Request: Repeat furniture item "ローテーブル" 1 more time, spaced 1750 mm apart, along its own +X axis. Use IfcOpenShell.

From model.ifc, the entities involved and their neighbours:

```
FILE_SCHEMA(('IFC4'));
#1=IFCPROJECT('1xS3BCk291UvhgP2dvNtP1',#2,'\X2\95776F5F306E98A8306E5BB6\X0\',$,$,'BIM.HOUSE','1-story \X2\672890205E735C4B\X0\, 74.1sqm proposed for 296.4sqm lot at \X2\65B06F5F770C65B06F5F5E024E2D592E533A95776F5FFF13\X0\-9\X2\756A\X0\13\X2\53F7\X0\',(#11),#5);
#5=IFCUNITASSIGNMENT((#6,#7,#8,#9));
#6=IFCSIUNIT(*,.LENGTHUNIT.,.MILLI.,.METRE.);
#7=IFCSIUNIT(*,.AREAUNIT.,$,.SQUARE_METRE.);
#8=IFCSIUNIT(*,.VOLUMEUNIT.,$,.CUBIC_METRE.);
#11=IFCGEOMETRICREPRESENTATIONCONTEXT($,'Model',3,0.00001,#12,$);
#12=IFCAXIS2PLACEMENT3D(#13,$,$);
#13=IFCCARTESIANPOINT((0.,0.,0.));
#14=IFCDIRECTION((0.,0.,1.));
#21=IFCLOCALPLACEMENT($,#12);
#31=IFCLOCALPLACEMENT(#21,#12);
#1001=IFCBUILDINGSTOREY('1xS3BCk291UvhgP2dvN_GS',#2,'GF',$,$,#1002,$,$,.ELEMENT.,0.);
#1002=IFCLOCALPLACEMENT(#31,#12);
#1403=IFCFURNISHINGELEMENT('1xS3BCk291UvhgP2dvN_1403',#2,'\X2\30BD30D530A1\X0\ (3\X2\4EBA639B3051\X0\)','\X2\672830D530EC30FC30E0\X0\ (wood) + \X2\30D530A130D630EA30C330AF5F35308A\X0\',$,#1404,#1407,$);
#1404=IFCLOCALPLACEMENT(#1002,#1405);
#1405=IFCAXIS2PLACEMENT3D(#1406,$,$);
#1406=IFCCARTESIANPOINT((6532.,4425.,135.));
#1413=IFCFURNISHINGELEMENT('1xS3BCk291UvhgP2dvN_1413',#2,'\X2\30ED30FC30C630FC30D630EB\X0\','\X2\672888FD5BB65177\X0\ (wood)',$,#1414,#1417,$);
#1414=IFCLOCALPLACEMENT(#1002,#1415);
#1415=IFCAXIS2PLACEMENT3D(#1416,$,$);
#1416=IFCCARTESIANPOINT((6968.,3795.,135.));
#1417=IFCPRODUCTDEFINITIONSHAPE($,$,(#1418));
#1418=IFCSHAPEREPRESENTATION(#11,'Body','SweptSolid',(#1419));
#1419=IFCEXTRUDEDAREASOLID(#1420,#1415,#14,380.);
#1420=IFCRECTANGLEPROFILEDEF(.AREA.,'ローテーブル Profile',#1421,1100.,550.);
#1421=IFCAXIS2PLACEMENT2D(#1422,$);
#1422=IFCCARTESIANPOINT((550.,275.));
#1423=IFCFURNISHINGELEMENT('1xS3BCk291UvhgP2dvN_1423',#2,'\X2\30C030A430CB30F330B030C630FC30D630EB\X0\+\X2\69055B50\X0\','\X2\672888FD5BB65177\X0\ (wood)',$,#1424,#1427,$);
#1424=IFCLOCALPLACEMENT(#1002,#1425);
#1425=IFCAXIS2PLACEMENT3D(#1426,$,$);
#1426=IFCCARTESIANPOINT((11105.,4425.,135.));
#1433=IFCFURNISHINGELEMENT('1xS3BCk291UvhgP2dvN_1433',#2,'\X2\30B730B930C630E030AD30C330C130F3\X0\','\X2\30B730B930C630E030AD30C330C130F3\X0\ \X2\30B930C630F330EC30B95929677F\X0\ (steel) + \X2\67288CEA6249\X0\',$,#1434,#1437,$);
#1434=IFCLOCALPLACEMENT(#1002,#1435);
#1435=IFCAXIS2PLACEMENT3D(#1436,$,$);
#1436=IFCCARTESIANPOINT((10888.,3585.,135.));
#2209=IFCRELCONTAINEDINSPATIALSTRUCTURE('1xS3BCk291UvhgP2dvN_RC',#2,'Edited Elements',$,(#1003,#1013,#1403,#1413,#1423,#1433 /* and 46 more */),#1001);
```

```python
import ifcopenshell
import ifcopenshell.api.geometry
import ifcopenshell.api.root
import ifcopenshell.util.element
import ifcopenshell.util.placement
import ifcopenshell.util.unit

model = ifcopenshell.open("model.ifc")
unit_scale = ifcopenshell.util.unit.calculate_unit_scale(model)


def reuse_history(source, copy):
    """copy_class also copies each property set's owner history, people and application; keep the originals."""
    for rel in copy.IsDefinedBy:
        if rel.is_a("IfcRelDefinesByProperties") and (history := rel.RelatingPropertyDefinition.OwnerHistory):
            rel.RelatingPropertyDefinition.OwnerHistory = source.OwnerHistory
            ifcopenshell.util.element.remove_deep2(model, history)


source = model.by_id(1413)
base = ifcopenshell.util.placement.get_local_placement(source.ObjectPlacement)
step = base[:3, 0] * 1.75 / unit_scale

for i in range(1, 2):
    copy = ifcopenshell.api.root.copy_class(model, product=source)
    copy.Representation = ifcopenshell.util.element.copy_deep(
        model, source.Representation, exclude=["IfcGeometricRepresentationContext", "IfcRepresentationMap"]
    )
    reuse_history(source, copy)
    matrix = base.copy()
    matrix[:3, 3] += i * step
    print("added at", matrix[:3, 3].round(3) + 0.0)
    ifcopenshell.api.geometry.edit_object_placement(model, product=copy, matrix=matrix, is_si=False)

model.write("model_v2.ifc")
```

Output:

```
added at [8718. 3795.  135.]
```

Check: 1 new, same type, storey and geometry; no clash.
